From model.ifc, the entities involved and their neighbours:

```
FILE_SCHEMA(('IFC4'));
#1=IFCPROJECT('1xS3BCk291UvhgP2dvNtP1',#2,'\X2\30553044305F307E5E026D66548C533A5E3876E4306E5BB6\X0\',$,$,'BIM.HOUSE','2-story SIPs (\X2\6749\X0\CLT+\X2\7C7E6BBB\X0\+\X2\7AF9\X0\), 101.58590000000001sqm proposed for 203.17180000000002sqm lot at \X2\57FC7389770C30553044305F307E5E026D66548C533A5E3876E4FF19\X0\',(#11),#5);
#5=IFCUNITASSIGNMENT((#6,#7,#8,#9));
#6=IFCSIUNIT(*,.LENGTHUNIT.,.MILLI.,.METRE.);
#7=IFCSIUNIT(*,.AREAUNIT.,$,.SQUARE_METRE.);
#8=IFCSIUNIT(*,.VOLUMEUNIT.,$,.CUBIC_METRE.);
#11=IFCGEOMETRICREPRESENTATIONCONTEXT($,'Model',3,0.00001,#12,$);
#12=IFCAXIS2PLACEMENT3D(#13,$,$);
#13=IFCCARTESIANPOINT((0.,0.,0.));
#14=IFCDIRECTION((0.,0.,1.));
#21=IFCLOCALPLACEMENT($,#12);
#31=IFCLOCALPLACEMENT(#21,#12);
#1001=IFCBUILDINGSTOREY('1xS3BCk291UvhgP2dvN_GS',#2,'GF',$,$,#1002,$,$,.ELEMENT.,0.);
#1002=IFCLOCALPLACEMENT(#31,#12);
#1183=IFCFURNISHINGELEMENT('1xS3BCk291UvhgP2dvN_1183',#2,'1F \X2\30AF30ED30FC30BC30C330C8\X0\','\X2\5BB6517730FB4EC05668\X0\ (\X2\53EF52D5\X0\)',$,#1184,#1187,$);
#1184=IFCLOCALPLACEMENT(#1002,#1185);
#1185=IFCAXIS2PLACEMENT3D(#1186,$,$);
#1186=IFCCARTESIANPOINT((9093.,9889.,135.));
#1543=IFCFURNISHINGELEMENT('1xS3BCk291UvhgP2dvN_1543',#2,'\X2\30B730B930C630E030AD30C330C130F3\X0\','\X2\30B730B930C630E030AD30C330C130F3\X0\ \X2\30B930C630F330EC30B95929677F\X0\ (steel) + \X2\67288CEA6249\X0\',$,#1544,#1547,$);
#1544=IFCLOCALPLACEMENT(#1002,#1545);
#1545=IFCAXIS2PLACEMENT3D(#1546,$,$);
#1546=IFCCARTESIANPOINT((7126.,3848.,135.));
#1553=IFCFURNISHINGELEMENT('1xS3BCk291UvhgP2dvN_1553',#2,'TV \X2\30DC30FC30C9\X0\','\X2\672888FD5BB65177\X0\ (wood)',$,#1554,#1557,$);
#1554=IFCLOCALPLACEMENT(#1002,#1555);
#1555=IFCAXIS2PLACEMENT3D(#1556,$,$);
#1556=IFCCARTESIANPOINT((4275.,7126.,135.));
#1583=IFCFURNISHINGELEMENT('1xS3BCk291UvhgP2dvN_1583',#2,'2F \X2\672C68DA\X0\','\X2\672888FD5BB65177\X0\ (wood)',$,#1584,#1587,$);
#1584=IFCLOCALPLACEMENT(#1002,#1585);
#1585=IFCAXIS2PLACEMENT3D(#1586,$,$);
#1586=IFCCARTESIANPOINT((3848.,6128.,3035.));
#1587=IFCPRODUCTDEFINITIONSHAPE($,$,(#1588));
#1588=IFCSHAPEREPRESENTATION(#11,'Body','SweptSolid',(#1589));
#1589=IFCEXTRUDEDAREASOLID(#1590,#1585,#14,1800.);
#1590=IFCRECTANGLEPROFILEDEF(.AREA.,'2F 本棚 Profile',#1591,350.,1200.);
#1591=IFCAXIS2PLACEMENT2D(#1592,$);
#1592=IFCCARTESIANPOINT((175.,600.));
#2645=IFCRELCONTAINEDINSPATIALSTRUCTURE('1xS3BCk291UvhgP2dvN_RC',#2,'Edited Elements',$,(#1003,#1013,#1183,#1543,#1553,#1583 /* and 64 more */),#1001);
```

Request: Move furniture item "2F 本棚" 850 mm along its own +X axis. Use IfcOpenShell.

```python
import ifcopenshell
import ifcopenshell.api.geometry
import ifcopenshell.util.placement

model = ifcopenshell.open("model.ifc")

item = model.by_guid("1xS3BCk291UvhgP2dvN_1583")
matrix = ifcopenshell.util.placement.get_local_placement(item.ObjectPlacement)
matrix[:3, 3] += matrix[:3, 0] * 850.0
ifcopenshell.api.geometry.edit_object_placement(model, product=item, matrix=matrix, is_si=False)

print(ifcopenshell.util.placement.get_local_placement(item.ObjectPlacement).round(3) + 0.0)

model.write("model_updated.ifc")
```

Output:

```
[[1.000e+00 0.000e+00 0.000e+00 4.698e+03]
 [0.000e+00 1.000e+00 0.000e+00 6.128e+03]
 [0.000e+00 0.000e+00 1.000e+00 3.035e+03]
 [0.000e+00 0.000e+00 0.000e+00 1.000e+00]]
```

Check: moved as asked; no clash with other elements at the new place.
